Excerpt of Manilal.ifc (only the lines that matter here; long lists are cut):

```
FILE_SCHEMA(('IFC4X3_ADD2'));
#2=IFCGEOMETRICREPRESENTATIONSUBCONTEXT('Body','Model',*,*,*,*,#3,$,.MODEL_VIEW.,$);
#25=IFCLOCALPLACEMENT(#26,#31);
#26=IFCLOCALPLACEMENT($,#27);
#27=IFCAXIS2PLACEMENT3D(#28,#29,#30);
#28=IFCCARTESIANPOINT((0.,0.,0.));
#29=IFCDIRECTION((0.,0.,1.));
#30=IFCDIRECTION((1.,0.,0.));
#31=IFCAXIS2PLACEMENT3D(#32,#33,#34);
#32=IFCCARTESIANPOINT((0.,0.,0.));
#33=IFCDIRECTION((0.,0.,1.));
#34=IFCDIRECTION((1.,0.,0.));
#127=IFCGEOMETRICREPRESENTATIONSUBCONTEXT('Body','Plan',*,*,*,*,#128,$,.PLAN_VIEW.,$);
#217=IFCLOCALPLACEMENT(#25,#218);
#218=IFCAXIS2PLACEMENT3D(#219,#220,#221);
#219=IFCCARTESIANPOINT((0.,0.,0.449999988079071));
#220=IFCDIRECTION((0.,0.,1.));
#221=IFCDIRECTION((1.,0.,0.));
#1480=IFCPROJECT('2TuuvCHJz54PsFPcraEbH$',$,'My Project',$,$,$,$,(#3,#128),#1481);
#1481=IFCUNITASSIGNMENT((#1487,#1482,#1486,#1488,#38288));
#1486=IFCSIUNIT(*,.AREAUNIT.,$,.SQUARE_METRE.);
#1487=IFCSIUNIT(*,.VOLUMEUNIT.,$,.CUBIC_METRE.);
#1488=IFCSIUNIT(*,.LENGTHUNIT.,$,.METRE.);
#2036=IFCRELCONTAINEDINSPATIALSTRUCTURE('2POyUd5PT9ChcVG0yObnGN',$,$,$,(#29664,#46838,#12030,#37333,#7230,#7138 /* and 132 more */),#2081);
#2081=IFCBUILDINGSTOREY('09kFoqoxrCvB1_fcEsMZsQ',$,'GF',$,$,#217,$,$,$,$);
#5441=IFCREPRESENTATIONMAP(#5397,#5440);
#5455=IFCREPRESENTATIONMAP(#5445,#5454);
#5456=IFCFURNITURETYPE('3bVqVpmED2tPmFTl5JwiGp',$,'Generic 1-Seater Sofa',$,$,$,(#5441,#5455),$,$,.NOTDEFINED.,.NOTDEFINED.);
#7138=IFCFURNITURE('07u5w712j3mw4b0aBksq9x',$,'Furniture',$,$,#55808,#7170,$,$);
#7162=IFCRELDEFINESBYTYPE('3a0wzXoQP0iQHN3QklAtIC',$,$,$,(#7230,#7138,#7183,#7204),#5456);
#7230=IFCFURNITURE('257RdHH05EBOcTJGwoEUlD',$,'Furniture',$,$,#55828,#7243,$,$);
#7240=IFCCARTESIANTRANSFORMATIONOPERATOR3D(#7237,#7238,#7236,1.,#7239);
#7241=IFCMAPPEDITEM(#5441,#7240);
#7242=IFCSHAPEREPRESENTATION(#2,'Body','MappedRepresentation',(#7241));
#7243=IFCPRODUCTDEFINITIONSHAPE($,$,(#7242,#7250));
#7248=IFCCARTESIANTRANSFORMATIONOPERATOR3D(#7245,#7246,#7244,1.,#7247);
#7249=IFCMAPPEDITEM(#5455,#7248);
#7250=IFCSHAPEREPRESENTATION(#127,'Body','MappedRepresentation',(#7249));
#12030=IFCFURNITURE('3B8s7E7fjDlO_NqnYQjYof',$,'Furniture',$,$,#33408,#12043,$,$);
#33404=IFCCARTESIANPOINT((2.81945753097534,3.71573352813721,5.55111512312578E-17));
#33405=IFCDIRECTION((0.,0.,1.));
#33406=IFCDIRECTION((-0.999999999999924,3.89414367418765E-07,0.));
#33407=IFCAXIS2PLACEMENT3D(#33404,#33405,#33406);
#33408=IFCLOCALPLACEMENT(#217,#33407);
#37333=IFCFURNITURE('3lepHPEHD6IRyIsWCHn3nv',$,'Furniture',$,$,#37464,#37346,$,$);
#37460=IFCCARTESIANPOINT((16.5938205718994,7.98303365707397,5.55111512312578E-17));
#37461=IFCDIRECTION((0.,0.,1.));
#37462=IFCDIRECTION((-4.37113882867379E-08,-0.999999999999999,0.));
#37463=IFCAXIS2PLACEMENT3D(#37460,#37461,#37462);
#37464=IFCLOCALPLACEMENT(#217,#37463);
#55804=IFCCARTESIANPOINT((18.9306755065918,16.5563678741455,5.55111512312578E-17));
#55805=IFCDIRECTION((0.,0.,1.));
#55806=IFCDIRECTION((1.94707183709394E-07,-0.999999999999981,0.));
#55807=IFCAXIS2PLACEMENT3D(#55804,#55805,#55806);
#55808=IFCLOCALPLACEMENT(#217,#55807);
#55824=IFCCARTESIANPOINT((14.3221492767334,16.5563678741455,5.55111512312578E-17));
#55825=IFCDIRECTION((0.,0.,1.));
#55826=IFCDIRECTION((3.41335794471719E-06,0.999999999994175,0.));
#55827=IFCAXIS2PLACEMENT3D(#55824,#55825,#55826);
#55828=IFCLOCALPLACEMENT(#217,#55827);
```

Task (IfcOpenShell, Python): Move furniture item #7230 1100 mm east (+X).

```python
import ifcopenshell
import ifcopenshell.api.geometry
import ifcopenshell.util.placement

model = ifcopenshell.open("Manilal.ifc")

item = model.by_guid("257RdHH05EBOcTJGwoEUlD")
matrix = ifcopenshell.util.placement.get_local_placement(item.ObjectPlacement)
matrix[0, 3] += 1.1
ifcopenshell.api.geometry.edit_object_placement(model, product=item, matrix=matrix, is_si=False)

print(ifcopenshell.util.placement.get_local_placement(item.ObjectPlacement).round(3) + 0.0)

model.write("Manilal_rev.ifc")
```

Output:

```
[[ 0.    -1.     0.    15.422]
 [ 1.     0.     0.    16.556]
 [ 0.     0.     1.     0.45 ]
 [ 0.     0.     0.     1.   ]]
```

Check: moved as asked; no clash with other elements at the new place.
